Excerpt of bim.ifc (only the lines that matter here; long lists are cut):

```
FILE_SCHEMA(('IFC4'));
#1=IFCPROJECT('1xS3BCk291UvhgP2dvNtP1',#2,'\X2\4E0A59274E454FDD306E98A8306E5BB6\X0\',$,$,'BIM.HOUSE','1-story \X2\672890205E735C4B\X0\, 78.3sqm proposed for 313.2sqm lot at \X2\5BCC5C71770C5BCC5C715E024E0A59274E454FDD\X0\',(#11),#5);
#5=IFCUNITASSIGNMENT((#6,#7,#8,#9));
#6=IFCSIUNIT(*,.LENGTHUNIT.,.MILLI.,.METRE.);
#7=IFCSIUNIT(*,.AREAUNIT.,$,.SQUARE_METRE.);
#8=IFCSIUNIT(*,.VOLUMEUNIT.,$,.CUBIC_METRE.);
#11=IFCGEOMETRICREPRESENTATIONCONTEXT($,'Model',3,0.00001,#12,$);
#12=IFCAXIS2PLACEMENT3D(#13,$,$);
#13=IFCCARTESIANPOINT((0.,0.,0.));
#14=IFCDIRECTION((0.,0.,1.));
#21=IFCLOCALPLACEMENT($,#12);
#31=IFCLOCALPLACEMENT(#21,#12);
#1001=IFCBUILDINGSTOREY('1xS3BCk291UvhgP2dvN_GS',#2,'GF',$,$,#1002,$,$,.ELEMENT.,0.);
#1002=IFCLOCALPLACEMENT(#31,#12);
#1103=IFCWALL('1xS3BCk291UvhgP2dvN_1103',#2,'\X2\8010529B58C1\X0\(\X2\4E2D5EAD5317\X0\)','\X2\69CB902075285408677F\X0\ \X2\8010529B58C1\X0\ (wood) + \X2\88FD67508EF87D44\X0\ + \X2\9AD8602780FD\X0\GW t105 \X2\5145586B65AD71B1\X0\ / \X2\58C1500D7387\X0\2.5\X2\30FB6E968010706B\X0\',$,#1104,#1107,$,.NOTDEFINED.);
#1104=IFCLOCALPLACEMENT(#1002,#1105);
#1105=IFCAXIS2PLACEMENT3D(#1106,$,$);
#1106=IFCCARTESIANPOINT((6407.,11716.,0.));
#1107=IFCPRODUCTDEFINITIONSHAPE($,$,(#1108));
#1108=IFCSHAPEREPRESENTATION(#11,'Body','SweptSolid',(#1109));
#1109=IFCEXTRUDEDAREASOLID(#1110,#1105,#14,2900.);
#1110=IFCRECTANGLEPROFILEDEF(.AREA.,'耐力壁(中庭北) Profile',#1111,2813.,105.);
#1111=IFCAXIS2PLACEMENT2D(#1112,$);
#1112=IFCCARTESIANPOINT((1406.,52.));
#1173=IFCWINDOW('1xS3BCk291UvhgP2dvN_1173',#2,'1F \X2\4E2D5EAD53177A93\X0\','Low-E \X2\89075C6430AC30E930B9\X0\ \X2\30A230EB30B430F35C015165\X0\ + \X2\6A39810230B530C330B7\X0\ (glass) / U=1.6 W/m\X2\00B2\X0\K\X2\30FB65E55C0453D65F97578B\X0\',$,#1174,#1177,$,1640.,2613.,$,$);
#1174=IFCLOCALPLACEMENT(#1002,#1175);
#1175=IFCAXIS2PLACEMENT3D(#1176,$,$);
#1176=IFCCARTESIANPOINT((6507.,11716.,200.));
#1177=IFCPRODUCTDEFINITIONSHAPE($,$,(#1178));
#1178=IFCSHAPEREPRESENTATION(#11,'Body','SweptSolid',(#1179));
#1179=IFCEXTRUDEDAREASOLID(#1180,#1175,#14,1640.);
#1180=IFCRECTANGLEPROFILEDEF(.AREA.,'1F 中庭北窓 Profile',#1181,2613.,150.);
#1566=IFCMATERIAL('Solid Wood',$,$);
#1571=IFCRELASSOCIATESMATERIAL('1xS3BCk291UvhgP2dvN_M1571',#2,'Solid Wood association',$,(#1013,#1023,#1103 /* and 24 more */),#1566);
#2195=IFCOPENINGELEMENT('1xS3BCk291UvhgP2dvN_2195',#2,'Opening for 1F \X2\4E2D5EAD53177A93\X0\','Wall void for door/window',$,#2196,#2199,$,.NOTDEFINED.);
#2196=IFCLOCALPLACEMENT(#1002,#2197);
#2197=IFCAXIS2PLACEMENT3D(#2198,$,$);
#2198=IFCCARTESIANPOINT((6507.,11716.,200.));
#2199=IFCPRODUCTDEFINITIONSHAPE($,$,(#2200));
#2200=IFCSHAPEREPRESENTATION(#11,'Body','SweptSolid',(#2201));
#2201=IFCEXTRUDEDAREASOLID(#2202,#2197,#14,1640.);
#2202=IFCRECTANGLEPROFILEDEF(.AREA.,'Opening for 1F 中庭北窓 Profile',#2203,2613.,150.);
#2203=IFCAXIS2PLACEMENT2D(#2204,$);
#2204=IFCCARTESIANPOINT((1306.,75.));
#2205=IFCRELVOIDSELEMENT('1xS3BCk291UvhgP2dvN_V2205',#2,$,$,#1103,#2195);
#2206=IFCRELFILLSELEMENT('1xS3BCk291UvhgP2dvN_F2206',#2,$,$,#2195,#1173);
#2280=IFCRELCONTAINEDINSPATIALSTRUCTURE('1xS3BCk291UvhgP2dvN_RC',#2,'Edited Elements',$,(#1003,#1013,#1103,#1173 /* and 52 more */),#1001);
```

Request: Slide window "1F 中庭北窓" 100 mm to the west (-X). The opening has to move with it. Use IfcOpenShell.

```python
import ifcopenshell
import ifcopenshell.api.geometry
import ifcopenshell.util.placement
import ifcopenshell.util.unit

model = ifcopenshell.open("bim.ifc")
unit_scale = ifcopenshell.util.unit.calculate_unit_scale(model)

window = model.by_guid("1xS3BCk291UvhgP2dvN_1173")
opening = window.FillsVoids[0].RelatingOpeningElement
wall = opening.VoidsElements[0].RelatingBuildingElement

wall_matrix = ifcopenshell.util.placement.get_local_placement(wall.ObjectPlacement)
shift = wall_matrix[:3, 0] * -0.1 / unit_scale
before = ifcopenshell.util.placement.get_local_placement(window.ObjectPlacement)[:3, 3].copy()

# The window is not placed relative to its opening, so move both.
for product in (opening, window):
    matrix = ifcopenshell.util.placement.get_local_placement(product.ObjectPlacement)
    matrix[:3, 3] += shift
    ifcopenshell.api.geometry.edit_object_placement(model, product=product, matrix=matrix, is_si=False)

after = ifcopenshell.util.placement.get_local_placement(window.ObjectPlacement)[:3, 3]
print("window moved by", (after - before).round(3) + 0.0)

model.write("bim_rev.ifc")
```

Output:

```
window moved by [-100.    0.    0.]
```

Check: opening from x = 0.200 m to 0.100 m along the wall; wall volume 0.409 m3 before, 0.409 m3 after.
